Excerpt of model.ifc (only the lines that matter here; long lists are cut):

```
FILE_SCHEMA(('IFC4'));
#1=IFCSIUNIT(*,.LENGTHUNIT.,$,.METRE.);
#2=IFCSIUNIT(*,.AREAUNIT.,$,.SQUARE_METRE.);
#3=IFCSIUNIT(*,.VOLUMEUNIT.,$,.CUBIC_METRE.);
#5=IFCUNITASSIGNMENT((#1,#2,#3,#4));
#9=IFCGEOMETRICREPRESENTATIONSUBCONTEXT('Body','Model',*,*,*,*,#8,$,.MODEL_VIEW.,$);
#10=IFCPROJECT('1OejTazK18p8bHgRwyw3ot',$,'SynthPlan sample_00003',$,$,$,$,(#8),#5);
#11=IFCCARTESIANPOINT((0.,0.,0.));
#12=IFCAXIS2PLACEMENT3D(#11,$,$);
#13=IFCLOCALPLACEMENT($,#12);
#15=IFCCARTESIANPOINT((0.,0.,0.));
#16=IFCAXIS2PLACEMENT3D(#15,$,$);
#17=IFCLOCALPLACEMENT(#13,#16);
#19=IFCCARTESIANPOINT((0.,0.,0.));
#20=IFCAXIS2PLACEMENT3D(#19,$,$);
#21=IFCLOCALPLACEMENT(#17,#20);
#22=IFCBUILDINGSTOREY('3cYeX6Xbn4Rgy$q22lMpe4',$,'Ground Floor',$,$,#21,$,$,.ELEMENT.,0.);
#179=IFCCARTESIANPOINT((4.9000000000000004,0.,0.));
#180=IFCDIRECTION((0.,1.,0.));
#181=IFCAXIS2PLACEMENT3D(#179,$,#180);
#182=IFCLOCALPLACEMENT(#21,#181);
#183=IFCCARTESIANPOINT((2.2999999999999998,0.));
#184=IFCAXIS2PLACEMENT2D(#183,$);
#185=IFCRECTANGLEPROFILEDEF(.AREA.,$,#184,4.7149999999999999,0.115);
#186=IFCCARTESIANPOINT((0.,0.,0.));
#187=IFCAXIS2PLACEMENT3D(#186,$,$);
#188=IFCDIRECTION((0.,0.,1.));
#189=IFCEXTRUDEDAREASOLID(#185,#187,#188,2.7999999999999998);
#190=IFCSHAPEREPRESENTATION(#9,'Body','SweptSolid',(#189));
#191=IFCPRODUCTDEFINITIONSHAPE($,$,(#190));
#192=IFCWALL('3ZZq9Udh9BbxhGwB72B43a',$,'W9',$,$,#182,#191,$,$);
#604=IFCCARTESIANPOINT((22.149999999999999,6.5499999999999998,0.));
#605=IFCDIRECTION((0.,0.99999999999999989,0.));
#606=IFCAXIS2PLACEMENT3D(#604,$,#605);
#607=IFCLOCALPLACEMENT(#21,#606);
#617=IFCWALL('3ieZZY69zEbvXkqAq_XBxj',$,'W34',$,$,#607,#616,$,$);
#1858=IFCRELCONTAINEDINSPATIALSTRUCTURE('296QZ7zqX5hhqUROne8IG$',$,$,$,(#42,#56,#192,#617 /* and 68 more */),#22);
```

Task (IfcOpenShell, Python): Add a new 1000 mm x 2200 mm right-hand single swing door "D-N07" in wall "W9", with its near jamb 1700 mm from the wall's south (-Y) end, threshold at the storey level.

```python
import numpy as np
import ifcopenshell
import ifcopenshell.api.feature
import ifcopenshell.api.geometry
import ifcopenshell.api.root
import ifcopenshell.api.spatial
import ifcopenshell.geom
import ifcopenshell.util.element
import ifcopenshell.util.placement
import ifcopenshell.util.representation
import ifcopenshell.util.shape
import ifcopenshell.util.unit

model = ifcopenshell.open("model.ifc")
unit_scale = ifcopenshell.util.unit.calculate_unit_scale(model)
settings = ifcopenshell.geom.settings()


def volume(element):
    """Net volume in cubic metres, openings subtracted."""
    shape = ifcopenshell.geom.create_shape(settings, element)
    return ifcopenshell.util.shape.get_volume(shape.geometry)


wall = model.by_guid("3ZZq9Udh9BbxhGwB72B43a")
storey = ifcopenshell.util.element.get_container(wall, ifc_class="IfcBuildingStorey")
context = ifcopenshell.util.representation.get_context(model, "Model", "Body", "MODEL_VIEW")
before = volume(wall)

width, height, from_end, sill = 1, 2.2, 1.7, 0.0  # metres

# The wall runs along its own X axis, and the end named is its -X end.
wall_shape = ifcopenshell.geom.create_shape(settings, wall)
x, y, z = ifcopenshell.util.shape.get_vertices(wall_shape.geometry).T
start = x.min() + from_end
face, thickness = float(y.min()), float(y.max() - y.min())
wall_matrix = ifcopenshell.util.placement.get_local_placement(wall.ObjectPlacement)
level = ifcopenshell.util.placement.get_local_placement(storey.ObjectPlacement)[2, 3]


def in_wall(x, y):
    """Placement at x, y metres in the wall's axes, at sill height."""
    matrix = wall_matrix.copy()
    matrix[:, 3] = wall_matrix @ np.array([x / unit_scale, y / unit_scale, 0.0, 1.0])
    matrix[2, 3] = level + sill / unit_scale
    return matrix


# Opening: a box that overshoots both wall faces by 50 mm.
opening = ifcopenshell.api.root.create_entity(model, ifc_class="IfcOpeningElement", predefined_type="OPENING")
box = ifcopenshell.api.geometry.add_wall_representation(
    model, context=context, length=width, height=height, thickness=thickness + 0.1
)
ifcopenshell.api.geometry.assign_representation(model, product=opening, representation=box)
ifcopenshell.api.geometry.edit_object_placement(model, product=opening, matrix=in_wall(start, face - 0.05), is_si=False)
ifcopenshell.api.feature.add_feature(model, feature=opening, element=wall)

door = ifcopenshell.api.root.create_entity(model, ifc_class="IfcDoor", name="D-N07", predefined_type="DOOR")
door.OverallWidth, door.OverallHeight = width / unit_scale, height / unit_scale
door.OperationType = "SINGLE_SWING_RIGHT"
body = ifcopenshell.api.geometry.add_door_representation(
    model,
    context=context,
    overall_width=door.OverallWidth,
    overall_height=door.OverallHeight,
    operation_type="SINGLE_SWING_RIGHT",
    lining_properties={"LiningDepth": thickness / unit_scale, "ThresholdDepth": thickness / unit_scale},
)
ifcopenshell.api.geometry.assign_representation(model, product=door, representation=body)
ifcopenshell.api.spatial.assign_container(model, products=[door], relating_structure=storey)
ifcopenshell.api.feature.add_filling(model, opening=opening, element=door)

# The lining spans the wall, so the door starts at the wall face.
ifcopenshell.api.geometry.edit_object_placement(model, product=door, matrix=in_wall(start, face), is_si=False)

after = volume(wall)

print(f"wall volume {before:.3f} -> {after:.3f} m3")

model.write("model_edited.ifc")
```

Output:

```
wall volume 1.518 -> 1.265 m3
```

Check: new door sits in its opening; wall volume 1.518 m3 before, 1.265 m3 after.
